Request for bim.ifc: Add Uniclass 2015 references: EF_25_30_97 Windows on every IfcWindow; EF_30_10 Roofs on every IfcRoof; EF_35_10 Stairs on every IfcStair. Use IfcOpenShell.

First a look at what the model holds.

```python
import ifcopenshell

model = ifcopenshell.open("bim.ifc")
print(model.schema)
print("classifications:", [c.Name for c in model.by_type("IfcClassification")])
for ifc_class in ("IfcDoor", "IfcRoof", "IfcStair", "IfcWall", "IfcWindow"):
    print(ifc_class, len(model.by_type(ifc_class)))
```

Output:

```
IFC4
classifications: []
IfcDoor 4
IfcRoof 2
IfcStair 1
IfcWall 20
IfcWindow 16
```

```python
import ifcopenshell
import ifcopenshell.api.classification

model = ifcopenshell.open("bim.ifc")

system = ifcopenshell.api.classification.add_classification(model, classification="Uniclass 2015")

codes = {
    "IfcWindow": ("EF_25_30_97", "Windows"),
    "IfcRoof": ("EF_30_10", "Roofs"),
    "IfcStair": ("EF_35_10", "Stairs"),
}
for ifc_class, (code, name) in codes.items():
    products = model.by_type(ifc_class)
    ifcopenshell.api.classification.add_reference(
        model, products=products, classification=system, identification=code, name=name
    )
    print(code, len(products))

model.write("bim_rev.ifc")
```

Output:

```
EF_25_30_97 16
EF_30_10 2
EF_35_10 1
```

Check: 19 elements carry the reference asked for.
